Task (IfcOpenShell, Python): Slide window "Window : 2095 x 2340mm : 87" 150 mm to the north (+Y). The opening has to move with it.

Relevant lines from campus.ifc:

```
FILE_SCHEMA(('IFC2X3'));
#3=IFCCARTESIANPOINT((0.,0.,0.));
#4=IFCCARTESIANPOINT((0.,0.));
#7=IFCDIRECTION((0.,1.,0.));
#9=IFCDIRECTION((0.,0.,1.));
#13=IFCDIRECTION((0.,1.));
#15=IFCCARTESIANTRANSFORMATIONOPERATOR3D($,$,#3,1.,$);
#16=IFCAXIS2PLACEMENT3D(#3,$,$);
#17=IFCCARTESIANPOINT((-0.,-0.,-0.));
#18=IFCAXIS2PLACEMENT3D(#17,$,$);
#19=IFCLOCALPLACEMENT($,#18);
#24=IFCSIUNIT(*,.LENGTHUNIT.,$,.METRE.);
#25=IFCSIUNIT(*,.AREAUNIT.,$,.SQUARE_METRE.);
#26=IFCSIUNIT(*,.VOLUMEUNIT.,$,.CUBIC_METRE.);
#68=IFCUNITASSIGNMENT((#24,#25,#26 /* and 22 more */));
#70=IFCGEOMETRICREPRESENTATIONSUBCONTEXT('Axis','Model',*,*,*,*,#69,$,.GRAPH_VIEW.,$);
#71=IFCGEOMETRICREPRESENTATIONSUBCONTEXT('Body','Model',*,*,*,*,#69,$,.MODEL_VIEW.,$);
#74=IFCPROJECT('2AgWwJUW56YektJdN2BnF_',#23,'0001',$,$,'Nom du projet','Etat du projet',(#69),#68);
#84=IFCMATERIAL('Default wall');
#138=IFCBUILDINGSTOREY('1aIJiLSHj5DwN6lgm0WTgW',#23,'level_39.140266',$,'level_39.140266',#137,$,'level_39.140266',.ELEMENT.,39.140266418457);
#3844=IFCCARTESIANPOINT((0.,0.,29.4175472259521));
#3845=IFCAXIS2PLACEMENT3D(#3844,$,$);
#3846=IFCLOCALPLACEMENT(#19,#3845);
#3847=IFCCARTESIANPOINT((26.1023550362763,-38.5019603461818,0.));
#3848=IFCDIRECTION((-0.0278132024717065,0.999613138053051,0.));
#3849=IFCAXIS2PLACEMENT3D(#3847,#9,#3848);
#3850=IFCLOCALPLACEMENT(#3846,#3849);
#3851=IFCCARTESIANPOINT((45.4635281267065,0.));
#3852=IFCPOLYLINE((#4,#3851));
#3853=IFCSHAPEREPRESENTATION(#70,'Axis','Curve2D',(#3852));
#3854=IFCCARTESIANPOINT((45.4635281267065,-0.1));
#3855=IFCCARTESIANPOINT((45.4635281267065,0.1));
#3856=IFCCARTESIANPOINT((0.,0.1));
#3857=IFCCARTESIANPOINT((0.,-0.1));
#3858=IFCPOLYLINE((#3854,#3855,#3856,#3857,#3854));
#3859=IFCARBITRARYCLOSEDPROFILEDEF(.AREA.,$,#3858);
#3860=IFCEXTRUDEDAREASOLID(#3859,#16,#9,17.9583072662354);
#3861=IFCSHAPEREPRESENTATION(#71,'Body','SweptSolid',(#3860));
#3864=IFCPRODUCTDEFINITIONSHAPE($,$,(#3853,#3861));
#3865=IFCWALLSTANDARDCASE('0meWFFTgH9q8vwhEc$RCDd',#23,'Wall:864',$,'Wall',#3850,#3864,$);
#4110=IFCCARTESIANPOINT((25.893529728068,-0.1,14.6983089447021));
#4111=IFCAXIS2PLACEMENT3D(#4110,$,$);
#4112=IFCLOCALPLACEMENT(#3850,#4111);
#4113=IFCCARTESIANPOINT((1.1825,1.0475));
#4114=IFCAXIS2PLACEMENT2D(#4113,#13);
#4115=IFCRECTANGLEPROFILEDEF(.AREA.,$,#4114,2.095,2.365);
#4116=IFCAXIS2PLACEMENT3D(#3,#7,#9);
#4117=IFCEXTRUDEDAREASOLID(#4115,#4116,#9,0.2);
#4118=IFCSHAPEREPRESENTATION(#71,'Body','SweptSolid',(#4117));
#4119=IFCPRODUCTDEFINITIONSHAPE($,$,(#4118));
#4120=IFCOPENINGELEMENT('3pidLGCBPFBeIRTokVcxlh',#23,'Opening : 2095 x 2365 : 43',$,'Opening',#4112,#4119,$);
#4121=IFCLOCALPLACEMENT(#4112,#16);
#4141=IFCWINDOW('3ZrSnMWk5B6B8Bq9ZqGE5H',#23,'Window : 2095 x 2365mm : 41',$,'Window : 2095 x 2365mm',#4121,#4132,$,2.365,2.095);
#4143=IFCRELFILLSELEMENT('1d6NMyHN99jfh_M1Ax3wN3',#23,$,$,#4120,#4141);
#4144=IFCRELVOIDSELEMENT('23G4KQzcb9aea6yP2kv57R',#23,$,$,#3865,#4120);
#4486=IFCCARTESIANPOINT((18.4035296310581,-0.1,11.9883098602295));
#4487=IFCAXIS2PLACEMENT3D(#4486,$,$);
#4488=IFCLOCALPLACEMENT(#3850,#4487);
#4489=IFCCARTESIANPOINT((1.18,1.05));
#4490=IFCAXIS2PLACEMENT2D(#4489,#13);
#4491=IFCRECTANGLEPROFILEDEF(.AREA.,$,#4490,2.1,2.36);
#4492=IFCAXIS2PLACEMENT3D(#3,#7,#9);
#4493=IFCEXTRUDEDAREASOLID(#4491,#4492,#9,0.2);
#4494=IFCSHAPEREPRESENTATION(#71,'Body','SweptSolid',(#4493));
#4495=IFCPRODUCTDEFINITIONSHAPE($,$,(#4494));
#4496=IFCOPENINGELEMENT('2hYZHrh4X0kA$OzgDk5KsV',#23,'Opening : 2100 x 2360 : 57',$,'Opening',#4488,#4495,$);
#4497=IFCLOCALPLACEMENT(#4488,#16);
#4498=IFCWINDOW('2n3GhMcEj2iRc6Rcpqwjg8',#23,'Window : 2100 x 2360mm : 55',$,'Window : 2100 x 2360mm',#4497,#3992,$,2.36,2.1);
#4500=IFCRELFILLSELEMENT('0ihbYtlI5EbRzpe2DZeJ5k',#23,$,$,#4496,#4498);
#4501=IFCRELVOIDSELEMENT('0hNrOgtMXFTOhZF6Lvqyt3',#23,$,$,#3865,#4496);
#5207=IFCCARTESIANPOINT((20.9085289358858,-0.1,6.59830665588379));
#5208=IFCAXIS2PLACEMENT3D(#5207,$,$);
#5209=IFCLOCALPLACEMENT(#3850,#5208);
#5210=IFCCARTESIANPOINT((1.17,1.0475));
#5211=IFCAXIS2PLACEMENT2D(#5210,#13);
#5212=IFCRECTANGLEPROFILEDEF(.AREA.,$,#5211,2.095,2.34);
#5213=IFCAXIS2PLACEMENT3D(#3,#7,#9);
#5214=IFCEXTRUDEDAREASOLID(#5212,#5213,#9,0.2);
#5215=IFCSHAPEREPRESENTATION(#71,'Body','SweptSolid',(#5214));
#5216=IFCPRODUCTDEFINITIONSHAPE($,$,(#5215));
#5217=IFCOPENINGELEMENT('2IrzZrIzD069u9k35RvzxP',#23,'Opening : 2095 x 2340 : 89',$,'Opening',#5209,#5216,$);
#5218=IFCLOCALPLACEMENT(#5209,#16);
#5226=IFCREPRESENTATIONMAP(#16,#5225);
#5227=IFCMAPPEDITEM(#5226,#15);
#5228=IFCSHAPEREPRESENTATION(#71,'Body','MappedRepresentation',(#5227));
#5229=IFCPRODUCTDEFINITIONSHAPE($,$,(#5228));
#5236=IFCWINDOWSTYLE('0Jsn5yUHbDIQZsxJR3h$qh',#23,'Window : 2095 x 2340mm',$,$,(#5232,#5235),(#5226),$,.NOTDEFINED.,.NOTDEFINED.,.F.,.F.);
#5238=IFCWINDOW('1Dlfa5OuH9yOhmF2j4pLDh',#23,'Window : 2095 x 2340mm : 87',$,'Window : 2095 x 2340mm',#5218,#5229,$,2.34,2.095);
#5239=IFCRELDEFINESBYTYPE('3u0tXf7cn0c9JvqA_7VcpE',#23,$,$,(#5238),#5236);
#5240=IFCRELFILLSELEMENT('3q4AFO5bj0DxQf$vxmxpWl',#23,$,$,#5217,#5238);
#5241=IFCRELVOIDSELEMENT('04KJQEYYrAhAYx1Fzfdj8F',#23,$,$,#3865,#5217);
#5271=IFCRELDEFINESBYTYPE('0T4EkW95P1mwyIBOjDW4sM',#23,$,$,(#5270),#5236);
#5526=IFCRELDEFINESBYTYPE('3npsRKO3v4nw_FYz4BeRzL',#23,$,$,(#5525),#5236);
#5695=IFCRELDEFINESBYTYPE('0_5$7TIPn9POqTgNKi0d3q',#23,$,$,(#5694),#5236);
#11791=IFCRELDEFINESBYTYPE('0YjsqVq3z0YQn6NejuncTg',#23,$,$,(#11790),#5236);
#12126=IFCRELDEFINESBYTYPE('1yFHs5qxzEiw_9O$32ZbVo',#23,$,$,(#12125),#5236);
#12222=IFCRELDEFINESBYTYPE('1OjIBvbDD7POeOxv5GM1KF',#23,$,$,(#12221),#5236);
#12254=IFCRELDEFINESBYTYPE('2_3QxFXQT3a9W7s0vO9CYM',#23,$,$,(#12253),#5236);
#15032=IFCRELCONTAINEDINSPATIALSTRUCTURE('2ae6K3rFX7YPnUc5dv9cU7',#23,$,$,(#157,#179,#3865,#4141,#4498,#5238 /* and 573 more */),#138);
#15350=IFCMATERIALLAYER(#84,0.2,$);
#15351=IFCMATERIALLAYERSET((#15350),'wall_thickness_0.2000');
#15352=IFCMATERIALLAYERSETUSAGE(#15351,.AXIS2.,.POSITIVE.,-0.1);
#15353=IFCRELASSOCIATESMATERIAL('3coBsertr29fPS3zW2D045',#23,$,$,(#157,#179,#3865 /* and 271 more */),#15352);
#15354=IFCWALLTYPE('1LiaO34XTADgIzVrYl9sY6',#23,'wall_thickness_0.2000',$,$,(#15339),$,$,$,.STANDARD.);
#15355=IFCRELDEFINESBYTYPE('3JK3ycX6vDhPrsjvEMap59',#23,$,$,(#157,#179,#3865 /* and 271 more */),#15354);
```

```python
import ifcopenshell
import ifcopenshell.api.geometry
import ifcopenshell.util.placement
import ifcopenshell.util.unit

model = ifcopenshell.open("campus.ifc")
unit_scale = ifcopenshell.util.unit.calculate_unit_scale(model)

window = model.by_guid("1Dlfa5OuH9yOhmF2j4pLDh")
opening = window.FillsVoids[0].RelatingOpeningElement
wall = opening.VoidsElements[0].RelatingBuildingElement

wall_matrix = ifcopenshell.util.placement.get_local_placement(wall.ObjectPlacement)
shift = wall_matrix[:3, 0] * 0.15 / unit_scale
before = ifcopenshell.util.placement.get_local_placement(window.ObjectPlacement)[:3, 3].copy()

# The window is placed relative to its opening, so it follows when the opening moves.
matrix = ifcopenshell.util.placement.get_local_placement(opening.ObjectPlacement)
matrix[:3, 3] += shift
ifcopenshell.api.geometry.edit_object_placement(
    model, product=opening, matrix=matrix, is_si=False, should_transform_children=True
)

after = ifcopenshell.util.placement.get_local_placement(window.ObjectPlacement)[:3, 3]
print("window moved by", (after - before).round(3) + 0.0)

model.write("campus-out.ifc")
```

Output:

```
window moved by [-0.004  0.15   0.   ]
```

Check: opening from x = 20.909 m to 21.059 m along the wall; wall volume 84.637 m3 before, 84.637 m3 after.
